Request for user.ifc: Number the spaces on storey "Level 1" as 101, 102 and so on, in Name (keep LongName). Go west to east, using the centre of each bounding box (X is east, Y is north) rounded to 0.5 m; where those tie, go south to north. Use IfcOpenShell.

First a look at what the model holds.

```python
import ifcopenshell
import ifcopenshell.util.element
import ifcopenshell.util.placement

model = ifcopenshell.open("user.ifc")
print(model.schema)
storey = next(s for s in model.by_type("IfcBuildingStorey") if s.Name == "Level 1")
spaces = [e for e in ifcopenshell.util.element.get_decomposition(storey) if e.is_a("IfcSpace")]
for e in sorted(spaces, key=lambda e: e.id()):
    origin = ifcopenshell.util.placement.get_local_placement(e.ObjectPlacement)[:3, 3]
    print(e.id(), e.Name, e.LongName, origin.round(2) + 0.0, sep=" | ")
```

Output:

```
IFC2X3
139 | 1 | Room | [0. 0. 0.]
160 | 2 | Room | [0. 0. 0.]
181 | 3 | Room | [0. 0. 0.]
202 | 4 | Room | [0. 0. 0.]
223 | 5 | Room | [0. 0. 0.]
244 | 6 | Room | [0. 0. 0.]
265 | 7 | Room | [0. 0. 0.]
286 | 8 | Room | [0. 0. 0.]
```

```python
import ifcopenshell
import ifcopenshell.geom
import ifcopenshell.util.element
import ifcopenshell.util.shape

model = ifcopenshell.open("user.ifc")
settings = ifcopenshell.geom.settings()
settings.set("use-world-coords", True)


def centre(element):
    shape = ifcopenshell.geom.create_shape(settings, element)
    return ifcopenshell.util.shape.get_bbox_centroid(shape.geometry)


storey = next(s for s in model.by_type("IfcBuildingStorey") if s.Name == "Level 1")
spaces = [e for e in ifcopenshell.util.element.get_decomposition(storey) if e.is_a("IfcSpace")]

# Insertion points can sit at a corner or the storey origin, so sort by the geometry (in metres).
centres = {e: centre(e) for e in spaces}
spaces.sort(key=lambda e: (round(centres[e][0] / 0.5), centres[e][1]))

for i, e in enumerate(spaces, start=1):
    number = f"1{i:02d}"
    e.Name = number
    print(e.id(), number)

model.write("user_updated.ifc")
```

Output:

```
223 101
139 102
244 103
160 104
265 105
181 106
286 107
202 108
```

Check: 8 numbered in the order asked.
